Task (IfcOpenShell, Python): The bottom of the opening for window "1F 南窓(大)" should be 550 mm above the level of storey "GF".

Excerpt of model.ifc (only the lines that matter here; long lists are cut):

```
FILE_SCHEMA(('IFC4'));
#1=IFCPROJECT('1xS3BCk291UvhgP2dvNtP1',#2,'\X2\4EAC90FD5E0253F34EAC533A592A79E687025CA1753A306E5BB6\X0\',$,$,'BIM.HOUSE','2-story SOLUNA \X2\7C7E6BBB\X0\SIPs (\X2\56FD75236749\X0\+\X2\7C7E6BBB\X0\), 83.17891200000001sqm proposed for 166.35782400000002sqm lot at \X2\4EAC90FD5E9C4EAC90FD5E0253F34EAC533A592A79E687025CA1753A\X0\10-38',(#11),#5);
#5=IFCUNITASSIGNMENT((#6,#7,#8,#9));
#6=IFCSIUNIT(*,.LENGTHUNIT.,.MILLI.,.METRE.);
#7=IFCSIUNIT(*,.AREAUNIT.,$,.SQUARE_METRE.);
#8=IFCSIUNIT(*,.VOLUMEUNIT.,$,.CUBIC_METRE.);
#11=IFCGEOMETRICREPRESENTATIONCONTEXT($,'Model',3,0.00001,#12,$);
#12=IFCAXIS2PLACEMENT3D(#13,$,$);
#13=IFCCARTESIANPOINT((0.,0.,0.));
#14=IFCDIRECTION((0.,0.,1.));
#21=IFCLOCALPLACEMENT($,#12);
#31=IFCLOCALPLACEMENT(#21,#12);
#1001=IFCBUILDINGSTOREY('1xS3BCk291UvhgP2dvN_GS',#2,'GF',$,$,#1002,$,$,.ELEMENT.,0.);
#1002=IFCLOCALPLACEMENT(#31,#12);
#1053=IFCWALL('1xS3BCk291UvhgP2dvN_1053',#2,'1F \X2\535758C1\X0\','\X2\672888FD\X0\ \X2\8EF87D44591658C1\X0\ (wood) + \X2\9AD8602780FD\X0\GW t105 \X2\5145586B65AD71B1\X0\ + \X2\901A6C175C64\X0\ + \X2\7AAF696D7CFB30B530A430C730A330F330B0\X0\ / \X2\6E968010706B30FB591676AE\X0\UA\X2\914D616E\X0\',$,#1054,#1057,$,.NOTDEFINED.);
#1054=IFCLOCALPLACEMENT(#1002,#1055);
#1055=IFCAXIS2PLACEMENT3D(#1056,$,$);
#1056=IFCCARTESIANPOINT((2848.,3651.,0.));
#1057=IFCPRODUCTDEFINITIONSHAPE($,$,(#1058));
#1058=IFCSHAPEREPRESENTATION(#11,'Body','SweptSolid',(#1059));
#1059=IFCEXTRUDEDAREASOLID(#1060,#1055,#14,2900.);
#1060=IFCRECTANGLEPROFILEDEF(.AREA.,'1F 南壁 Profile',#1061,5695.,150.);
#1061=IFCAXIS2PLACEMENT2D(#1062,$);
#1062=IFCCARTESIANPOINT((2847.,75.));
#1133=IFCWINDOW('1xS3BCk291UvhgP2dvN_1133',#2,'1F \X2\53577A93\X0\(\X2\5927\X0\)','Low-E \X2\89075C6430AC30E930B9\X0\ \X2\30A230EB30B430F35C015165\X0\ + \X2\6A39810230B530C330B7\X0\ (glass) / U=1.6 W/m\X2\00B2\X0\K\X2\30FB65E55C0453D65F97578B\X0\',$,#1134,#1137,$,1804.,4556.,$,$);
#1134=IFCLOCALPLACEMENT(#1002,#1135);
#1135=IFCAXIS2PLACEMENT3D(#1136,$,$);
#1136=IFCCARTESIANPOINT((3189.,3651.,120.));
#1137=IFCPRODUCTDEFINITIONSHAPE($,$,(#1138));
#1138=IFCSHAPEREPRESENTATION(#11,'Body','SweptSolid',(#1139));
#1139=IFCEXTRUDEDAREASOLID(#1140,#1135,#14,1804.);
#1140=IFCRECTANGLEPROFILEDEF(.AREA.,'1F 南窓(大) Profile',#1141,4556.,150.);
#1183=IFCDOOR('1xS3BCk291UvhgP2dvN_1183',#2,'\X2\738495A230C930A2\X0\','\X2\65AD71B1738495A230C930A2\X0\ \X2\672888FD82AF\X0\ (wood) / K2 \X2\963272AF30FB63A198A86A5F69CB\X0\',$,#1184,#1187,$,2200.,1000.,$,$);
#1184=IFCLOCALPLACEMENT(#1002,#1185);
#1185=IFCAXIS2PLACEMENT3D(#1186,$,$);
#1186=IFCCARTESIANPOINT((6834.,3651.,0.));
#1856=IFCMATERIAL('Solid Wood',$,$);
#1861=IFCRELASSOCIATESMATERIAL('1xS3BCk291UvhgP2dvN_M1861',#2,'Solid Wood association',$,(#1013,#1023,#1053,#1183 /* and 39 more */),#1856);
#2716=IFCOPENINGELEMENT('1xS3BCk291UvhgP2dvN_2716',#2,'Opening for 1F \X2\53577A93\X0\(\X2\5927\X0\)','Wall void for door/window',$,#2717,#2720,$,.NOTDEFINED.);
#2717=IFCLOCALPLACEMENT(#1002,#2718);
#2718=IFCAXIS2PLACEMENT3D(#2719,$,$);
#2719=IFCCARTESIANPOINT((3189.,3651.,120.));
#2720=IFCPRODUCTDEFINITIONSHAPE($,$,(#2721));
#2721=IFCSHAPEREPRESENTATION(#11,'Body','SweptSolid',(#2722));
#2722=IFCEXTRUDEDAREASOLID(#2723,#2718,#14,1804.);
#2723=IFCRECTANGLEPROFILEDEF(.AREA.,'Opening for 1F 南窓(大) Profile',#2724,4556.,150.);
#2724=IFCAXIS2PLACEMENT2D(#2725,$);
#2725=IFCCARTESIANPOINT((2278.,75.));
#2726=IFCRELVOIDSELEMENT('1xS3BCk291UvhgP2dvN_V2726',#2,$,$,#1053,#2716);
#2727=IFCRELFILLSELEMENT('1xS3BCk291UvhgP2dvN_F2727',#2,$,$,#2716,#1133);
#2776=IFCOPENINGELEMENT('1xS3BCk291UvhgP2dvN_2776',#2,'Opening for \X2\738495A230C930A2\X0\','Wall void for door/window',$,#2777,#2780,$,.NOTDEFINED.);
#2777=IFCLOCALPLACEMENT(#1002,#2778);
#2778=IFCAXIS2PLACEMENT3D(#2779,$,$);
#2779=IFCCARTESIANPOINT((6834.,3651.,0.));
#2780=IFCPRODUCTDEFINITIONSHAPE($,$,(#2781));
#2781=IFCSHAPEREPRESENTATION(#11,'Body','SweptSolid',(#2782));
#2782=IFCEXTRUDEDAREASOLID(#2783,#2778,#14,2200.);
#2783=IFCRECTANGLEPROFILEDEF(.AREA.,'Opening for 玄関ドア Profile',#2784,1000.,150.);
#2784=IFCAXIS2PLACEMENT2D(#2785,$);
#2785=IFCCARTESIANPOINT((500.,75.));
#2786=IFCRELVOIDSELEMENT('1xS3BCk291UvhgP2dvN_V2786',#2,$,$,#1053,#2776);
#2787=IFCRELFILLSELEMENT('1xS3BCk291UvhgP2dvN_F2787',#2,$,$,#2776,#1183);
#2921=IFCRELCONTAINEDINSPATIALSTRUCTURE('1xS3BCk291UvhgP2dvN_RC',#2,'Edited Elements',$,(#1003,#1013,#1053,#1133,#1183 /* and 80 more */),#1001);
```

```python
import numpy as np
import ifcopenshell
import ifcopenshell.api.geometry
import ifcopenshell.geom
import ifcopenshell.util.element
import ifcopenshell.util.placement
import ifcopenshell.util.shape
import ifcopenshell.util.unit

model = ifcopenshell.open("model.ifc")
unit_scale = ifcopenshell.util.unit.calculate_unit_scale(model)

window = model.by_id(1133)
opening = window.FillsVoids[0].RelatingOpeningElement
storey = ifcopenshell.util.element.get_container(window, ifc_class="IfcBuildingStorey")
level = ifcopenshell.util.placement.get_local_placement(storey.ObjectPlacement)[2, 3]

# The opening's origin need not be at the sill, so measure its lowest point.
shape = ifcopenshell.geom.create_shape(ifcopenshell.geom.settings(), opening)
bottom = ifcopenshell.util.shape.get_shape_bottom_elevation(shape, shape.geometry) / unit_scale
dz = level + 550.0 - bottom

shift = np.array([0.0, 0.0, dz])
# The window is not placed relative to its opening, so move both.
for product in (opening, window):
    matrix = ifcopenshell.util.placement.get_local_placement(product.ObjectPlacement)
    matrix[:3, 3] += shift
    ifcopenshell.api.geometry.edit_object_placement(model, product=product, matrix=matrix, is_si=False)

print(f"moved by {dz * unit_scale:+.3f} m")

model.write("model_v2.ifc")
```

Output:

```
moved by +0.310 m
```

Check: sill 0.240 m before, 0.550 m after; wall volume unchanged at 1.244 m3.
